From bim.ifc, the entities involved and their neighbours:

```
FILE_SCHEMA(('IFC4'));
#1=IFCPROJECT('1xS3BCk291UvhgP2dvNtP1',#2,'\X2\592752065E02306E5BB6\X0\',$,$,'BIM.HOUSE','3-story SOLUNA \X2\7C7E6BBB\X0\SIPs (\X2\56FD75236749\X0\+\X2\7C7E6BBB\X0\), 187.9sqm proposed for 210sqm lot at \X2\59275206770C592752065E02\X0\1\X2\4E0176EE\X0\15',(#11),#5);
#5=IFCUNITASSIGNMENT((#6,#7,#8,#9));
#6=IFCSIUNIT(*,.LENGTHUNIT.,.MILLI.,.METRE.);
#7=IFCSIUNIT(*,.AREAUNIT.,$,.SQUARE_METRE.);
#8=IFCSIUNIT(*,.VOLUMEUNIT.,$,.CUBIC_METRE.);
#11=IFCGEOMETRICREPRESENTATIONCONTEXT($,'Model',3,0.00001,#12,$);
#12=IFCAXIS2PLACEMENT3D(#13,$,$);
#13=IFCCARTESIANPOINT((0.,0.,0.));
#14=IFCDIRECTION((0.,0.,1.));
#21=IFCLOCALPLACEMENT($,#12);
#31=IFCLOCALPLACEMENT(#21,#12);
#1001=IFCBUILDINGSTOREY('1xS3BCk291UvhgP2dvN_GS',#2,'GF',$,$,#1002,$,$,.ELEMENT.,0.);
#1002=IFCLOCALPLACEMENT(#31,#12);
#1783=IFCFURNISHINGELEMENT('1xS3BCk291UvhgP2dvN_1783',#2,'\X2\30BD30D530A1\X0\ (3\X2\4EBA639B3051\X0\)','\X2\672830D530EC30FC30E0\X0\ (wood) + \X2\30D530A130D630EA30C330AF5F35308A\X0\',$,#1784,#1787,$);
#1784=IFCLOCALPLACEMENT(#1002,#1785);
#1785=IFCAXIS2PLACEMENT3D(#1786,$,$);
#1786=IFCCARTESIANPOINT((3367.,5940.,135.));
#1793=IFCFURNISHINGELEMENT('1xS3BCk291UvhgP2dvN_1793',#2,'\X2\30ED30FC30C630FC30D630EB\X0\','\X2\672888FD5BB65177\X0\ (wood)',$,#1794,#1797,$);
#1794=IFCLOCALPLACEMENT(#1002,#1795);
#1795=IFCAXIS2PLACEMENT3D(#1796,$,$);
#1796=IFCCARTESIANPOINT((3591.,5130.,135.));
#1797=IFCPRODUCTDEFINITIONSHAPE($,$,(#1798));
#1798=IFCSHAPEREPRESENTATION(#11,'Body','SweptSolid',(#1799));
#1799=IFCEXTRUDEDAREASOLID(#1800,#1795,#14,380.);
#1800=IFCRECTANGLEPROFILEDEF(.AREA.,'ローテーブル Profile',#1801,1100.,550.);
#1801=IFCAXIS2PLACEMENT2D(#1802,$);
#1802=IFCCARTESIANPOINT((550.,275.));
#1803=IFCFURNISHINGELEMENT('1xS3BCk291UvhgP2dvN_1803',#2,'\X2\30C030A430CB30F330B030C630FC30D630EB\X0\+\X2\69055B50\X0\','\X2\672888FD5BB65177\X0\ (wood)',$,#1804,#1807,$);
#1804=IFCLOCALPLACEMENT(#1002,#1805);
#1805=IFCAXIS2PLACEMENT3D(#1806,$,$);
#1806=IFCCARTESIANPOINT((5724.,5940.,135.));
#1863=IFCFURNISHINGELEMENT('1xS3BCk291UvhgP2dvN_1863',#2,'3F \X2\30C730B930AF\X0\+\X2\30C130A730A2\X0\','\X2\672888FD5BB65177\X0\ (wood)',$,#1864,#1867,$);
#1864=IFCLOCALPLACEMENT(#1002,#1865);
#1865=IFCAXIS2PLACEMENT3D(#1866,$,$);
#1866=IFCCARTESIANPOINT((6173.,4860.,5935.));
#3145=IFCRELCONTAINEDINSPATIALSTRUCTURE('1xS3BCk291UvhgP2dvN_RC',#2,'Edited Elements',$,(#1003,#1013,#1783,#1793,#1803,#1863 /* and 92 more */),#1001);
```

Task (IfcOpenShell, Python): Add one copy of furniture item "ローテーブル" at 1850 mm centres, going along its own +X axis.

```python
import ifcopenshell
import ifcopenshell.api.geometry
import ifcopenshell.api.root
import ifcopenshell.util.element
import ifcopenshell.util.placement
import ifcopenshell.util.unit

model = ifcopenshell.open("bim.ifc")
unit_scale = ifcopenshell.util.unit.calculate_unit_scale(model)


def reuse_history(source, copy):
    """copy_class also copies each property set's owner history, people and application; keep the originals."""
    for rel in copy.IsDefinedBy:
        if rel.is_a("IfcRelDefinesByProperties") and (history := rel.RelatingPropertyDefinition.OwnerHistory):
            rel.RelatingPropertyDefinition.OwnerHistory = source.OwnerHistory
            ifcopenshell.util.element.remove_deep2(model, history)


source = model.by_id(1793)
base = ifcopenshell.util.placement.get_local_placement(source.ObjectPlacement)
step = base[:3, 0] * 1.85 / unit_scale

for i in range(1, 2):
    copy = ifcopenshell.api.root.copy_class(model, product=source)
    copy.Representation = ifcopenshell.util.element.copy_deep(
        model, source.Representation, exclude=["IfcGeometricRepresentationContext", "IfcRepresentationMap"]
    )
    reuse_history(source, copy)
    matrix = base.copy()
    matrix[:3, 3] += i * step
    print("added at", matrix[:3, 3].round(3) + 0.0)
    ifcopenshell.api.geometry.edit_object_placement(model, product=copy, matrix=matrix, is_si=False)

model.write("bim_v2.ifc")
```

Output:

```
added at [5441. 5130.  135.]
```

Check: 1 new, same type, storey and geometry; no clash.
